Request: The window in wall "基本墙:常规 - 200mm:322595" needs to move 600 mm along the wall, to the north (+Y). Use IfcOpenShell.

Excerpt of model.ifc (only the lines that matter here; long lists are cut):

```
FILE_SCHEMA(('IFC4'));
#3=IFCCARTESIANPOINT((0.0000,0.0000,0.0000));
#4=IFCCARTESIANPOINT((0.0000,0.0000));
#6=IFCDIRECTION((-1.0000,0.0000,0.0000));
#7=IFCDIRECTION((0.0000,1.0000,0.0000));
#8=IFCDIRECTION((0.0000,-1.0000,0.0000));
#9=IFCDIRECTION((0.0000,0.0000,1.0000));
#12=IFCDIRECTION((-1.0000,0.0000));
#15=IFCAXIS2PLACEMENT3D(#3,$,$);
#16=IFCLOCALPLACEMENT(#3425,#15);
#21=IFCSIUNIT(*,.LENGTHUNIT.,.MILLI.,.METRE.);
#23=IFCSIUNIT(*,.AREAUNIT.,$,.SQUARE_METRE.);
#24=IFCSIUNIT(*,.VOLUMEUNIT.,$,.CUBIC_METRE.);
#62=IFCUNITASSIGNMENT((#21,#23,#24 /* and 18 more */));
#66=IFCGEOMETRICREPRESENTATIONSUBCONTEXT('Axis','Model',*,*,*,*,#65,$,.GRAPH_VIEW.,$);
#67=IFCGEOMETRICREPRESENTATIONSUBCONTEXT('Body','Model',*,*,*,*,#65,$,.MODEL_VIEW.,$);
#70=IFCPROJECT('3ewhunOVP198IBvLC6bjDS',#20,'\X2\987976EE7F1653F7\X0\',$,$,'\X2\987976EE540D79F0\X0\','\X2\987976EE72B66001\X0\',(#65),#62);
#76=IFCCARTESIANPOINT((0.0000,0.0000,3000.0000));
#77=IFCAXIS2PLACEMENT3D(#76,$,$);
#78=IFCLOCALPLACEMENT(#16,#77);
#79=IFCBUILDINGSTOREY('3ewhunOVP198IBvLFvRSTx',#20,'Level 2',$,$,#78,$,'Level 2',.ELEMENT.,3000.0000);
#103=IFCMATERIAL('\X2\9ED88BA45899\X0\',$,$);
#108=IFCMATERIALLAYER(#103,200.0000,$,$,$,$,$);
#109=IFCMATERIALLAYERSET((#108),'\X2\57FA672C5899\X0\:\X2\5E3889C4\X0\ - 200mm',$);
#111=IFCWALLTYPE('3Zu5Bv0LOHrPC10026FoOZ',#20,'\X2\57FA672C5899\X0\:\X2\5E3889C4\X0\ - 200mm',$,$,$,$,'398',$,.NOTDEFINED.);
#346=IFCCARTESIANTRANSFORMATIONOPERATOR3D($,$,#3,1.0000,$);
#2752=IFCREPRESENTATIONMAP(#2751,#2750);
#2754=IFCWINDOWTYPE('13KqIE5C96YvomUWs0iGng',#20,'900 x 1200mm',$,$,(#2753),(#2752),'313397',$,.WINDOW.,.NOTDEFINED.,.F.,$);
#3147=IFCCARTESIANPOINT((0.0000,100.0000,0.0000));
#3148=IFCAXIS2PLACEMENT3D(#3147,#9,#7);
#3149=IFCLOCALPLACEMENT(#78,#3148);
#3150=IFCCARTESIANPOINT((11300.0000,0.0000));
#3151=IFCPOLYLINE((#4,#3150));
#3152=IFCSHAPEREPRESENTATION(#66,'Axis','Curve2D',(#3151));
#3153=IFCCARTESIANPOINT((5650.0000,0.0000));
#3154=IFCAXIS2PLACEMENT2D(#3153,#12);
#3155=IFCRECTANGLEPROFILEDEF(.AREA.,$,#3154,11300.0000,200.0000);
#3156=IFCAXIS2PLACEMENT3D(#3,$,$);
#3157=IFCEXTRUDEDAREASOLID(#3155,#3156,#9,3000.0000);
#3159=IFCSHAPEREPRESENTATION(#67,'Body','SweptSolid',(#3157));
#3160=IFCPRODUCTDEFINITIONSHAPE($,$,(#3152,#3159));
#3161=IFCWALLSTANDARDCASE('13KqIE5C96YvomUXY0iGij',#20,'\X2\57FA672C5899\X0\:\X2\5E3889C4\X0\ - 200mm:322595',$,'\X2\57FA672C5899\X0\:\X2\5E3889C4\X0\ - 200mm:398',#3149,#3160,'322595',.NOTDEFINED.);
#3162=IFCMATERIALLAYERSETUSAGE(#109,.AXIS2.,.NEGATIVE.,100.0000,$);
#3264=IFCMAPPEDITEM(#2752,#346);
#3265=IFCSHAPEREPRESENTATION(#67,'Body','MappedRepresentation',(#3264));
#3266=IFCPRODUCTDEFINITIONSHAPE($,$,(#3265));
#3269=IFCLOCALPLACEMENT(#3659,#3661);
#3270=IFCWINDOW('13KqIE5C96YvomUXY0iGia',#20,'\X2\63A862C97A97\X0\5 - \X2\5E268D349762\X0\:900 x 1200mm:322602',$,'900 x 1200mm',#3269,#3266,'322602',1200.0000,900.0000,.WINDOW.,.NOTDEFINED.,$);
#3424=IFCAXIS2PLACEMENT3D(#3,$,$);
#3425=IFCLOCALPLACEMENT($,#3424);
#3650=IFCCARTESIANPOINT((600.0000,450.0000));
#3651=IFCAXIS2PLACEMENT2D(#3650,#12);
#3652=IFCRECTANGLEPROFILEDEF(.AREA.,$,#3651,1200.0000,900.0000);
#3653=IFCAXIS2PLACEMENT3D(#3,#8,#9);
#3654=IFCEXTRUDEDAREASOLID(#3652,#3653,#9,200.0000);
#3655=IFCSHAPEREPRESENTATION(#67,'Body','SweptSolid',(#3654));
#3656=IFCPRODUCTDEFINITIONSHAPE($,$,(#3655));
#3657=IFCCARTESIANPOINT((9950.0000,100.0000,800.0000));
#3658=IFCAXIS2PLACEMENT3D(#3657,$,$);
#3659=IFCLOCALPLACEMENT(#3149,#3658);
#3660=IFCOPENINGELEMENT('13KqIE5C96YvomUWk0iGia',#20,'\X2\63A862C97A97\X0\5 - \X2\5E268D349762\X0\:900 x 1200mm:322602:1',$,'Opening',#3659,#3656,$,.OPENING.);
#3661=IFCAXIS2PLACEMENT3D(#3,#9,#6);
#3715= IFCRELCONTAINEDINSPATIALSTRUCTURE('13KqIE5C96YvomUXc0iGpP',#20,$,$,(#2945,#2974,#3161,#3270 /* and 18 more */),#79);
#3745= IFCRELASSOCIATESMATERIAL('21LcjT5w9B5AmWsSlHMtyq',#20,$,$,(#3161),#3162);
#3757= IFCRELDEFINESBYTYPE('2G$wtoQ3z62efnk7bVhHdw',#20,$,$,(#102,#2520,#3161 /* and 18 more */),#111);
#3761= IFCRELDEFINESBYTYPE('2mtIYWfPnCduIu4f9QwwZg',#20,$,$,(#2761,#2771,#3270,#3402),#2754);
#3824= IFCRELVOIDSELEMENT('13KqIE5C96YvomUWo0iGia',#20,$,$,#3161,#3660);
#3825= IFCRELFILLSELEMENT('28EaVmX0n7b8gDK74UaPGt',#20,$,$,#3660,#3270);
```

```python
import ifcopenshell
import ifcopenshell.api.geometry
import ifcopenshell.util.placement

model = ifcopenshell.open("model.ifc")

window = model.by_id(3270)
opening = window.FillsVoids[0].RelatingOpeningElement
wall = opening.VoidsElements[0].RelatingBuildingElement

wall_matrix = ifcopenshell.util.placement.get_local_placement(wall.ObjectPlacement)
shift = wall_matrix[:3, 0] * 600.0
before = ifcopenshell.util.placement.get_local_placement(window.ObjectPlacement)[:3, 3].copy()

# The window is placed relative to its opening, so it follows when the opening moves.
matrix = ifcopenshell.util.placement.get_local_placement(opening.ObjectPlacement)
matrix[:3, 3] += shift
ifcopenshell.api.geometry.edit_object_placement(
    model, product=opening, matrix=matrix, is_si=False, should_transform_children=True
)

after = ifcopenshell.util.placement.get_local_placement(window.ObjectPlacement)[:3, 3]
print("window moved by", (after - before).round(3) + 0.0)

model.write("model_updated.ifc")
```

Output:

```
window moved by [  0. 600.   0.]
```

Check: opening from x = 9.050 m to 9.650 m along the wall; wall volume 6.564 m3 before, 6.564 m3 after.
